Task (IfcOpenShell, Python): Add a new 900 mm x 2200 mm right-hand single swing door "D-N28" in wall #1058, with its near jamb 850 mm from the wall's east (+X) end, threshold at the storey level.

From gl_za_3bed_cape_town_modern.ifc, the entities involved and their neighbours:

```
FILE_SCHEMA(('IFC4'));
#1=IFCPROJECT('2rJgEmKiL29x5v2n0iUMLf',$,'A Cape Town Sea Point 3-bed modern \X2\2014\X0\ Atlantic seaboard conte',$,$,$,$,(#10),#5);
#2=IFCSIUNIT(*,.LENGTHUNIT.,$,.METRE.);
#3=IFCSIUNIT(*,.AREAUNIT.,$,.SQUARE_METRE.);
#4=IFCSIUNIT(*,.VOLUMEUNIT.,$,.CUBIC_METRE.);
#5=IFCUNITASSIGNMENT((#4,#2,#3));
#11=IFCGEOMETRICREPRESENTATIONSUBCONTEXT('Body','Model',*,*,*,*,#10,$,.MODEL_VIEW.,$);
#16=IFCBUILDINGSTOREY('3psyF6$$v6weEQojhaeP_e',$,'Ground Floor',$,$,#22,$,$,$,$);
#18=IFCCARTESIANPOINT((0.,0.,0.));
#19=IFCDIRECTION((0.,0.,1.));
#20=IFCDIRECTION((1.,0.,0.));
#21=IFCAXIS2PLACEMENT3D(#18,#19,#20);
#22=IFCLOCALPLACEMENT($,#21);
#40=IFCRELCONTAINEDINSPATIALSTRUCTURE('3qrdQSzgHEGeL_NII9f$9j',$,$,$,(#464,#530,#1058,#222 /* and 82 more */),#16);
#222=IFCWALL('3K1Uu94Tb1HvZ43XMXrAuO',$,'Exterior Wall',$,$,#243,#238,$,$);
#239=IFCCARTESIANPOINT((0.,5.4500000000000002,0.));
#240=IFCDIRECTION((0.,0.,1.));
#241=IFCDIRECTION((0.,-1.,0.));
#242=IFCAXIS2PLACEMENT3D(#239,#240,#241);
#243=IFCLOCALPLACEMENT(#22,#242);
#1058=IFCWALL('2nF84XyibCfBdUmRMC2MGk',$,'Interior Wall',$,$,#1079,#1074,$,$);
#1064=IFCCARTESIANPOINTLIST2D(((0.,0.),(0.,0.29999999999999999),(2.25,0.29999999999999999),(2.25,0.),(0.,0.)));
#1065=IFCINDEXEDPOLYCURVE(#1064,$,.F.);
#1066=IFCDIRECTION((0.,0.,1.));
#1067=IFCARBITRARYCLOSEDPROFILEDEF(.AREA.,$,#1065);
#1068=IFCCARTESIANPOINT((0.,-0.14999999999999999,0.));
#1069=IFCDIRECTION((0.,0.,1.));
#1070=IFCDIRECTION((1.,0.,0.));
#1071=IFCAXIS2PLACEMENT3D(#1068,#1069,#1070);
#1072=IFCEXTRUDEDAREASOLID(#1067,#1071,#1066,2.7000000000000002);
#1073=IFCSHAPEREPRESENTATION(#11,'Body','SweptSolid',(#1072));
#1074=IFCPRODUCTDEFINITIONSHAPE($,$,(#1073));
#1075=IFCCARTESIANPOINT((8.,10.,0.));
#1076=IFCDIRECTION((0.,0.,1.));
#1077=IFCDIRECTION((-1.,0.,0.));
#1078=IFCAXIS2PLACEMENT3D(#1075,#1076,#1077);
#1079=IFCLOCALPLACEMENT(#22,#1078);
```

```python
import numpy as np
import ifcopenshell
import ifcopenshell.api.feature
import ifcopenshell.api.geometry
import ifcopenshell.api.root
import ifcopenshell.api.spatial
import ifcopenshell.geom
import ifcopenshell.util.element
import ifcopenshell.util.placement
import ifcopenshell.util.representation
import ifcopenshell.util.shape
import ifcopenshell.util.unit

model = ifcopenshell.open("gl_za_3bed_cape_town_modern.ifc")
unit_scale = ifcopenshell.util.unit.calculate_unit_scale(model)
settings = ifcopenshell.geom.settings()


def volume(element):
    """Net volume in cubic metres, openings subtracted."""
    shape = ifcopenshell.geom.create_shape(settings, element)
    return ifcopenshell.util.shape.get_volume(shape.geometry)


wall = model.by_guid("2nF84XyibCfBdUmRMC2MGk")
storey = ifcopenshell.util.element.get_container(wall, ifc_class="IfcBuildingStorey")
context = ifcopenshell.util.representation.get_context(model, "Model", "Body", "MODEL_VIEW")
before = volume(wall)

width, height, from_end, sill = 0.9, 2.2, 0.85, 0.0  # metres

# The wall runs along its own X axis, and the end named is its -X end.
wall_shape = ifcopenshell.geom.create_shape(settings, wall)
x, y, z = ifcopenshell.util.shape.get_vertices(wall_shape.geometry).T
start = x.min() + from_end
face, thickness = float(y.min()), float(y.max() - y.min())
wall_matrix = ifcopenshell.util.placement.get_local_placement(wall.ObjectPlacement)
level = ifcopenshell.util.placement.get_local_placement(storey.ObjectPlacement)[2, 3]


def in_wall(x, y):
    """Placement at x, y metres in the wall's axes, at sill height."""
    matrix = wall_matrix.copy()
    matrix[:, 3] = wall_matrix @ np.array([x / unit_scale, y / unit_scale, 0.0, 1.0])
    matrix[2, 3] = level + sill / unit_scale
    return matrix


# Opening: a box that overshoots both wall faces by 50 mm.
opening = ifcopenshell.api.root.create_entity(model, ifc_class="IfcOpeningElement", predefined_type="OPENING")
box = ifcopenshell.api.geometry.add_wall_representation(
    model, context=context, length=width, height=height, thickness=thickness + 0.1
)
ifcopenshell.api.geometry.assign_representation(model, product=opening, representation=box)
ifcopenshell.api.geometry.edit_object_placement(model, product=opening, matrix=in_wall(start, face - 0.05), is_si=False)
ifcopenshell.api.feature.add_feature(model, feature=opening, element=wall)

door = ifcopenshell.api.root.create_entity(model, ifc_class="IfcDoor", name="D-N28", predefined_type="DOOR")
door.OverallWidth, door.OverallHeight = width / unit_scale, height / unit_scale
door.OperationType = "SINGLE_SWING_RIGHT"
body = ifcopenshell.api.geometry.add_door_representation(
    model,
    context=context,
    overall_width=door.OverallWidth,
    overall_height=door.OverallHeight,
    operation_type="SINGLE_SWING_RIGHT",
    lining_properties={"LiningDepth": thickness / unit_scale, "ThresholdDepth": thickness / unit_scale},
)
ifcopenshell.api.geometry.assign_representation(model, product=door, representation=body)
ifcopenshell.api.spatial.assign_container(model, products=[door], relating_structure=storey)
ifcopenshell.api.feature.add_filling(model, opening=opening, element=door)

# The lining spans the wall, so the door starts at the wall face.
ifcopenshell.api.geometry.edit_object_placement(model, product=door, matrix=in_wall(start, face), is_si=False)

after = volume(wall)

print(f"wall volume {before:.3f} -> {after:.3f} m3")

model.write("gl_za_3bed_cape_town_modern_rev.ifc")
```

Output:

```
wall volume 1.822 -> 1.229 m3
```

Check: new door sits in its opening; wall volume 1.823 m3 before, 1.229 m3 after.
